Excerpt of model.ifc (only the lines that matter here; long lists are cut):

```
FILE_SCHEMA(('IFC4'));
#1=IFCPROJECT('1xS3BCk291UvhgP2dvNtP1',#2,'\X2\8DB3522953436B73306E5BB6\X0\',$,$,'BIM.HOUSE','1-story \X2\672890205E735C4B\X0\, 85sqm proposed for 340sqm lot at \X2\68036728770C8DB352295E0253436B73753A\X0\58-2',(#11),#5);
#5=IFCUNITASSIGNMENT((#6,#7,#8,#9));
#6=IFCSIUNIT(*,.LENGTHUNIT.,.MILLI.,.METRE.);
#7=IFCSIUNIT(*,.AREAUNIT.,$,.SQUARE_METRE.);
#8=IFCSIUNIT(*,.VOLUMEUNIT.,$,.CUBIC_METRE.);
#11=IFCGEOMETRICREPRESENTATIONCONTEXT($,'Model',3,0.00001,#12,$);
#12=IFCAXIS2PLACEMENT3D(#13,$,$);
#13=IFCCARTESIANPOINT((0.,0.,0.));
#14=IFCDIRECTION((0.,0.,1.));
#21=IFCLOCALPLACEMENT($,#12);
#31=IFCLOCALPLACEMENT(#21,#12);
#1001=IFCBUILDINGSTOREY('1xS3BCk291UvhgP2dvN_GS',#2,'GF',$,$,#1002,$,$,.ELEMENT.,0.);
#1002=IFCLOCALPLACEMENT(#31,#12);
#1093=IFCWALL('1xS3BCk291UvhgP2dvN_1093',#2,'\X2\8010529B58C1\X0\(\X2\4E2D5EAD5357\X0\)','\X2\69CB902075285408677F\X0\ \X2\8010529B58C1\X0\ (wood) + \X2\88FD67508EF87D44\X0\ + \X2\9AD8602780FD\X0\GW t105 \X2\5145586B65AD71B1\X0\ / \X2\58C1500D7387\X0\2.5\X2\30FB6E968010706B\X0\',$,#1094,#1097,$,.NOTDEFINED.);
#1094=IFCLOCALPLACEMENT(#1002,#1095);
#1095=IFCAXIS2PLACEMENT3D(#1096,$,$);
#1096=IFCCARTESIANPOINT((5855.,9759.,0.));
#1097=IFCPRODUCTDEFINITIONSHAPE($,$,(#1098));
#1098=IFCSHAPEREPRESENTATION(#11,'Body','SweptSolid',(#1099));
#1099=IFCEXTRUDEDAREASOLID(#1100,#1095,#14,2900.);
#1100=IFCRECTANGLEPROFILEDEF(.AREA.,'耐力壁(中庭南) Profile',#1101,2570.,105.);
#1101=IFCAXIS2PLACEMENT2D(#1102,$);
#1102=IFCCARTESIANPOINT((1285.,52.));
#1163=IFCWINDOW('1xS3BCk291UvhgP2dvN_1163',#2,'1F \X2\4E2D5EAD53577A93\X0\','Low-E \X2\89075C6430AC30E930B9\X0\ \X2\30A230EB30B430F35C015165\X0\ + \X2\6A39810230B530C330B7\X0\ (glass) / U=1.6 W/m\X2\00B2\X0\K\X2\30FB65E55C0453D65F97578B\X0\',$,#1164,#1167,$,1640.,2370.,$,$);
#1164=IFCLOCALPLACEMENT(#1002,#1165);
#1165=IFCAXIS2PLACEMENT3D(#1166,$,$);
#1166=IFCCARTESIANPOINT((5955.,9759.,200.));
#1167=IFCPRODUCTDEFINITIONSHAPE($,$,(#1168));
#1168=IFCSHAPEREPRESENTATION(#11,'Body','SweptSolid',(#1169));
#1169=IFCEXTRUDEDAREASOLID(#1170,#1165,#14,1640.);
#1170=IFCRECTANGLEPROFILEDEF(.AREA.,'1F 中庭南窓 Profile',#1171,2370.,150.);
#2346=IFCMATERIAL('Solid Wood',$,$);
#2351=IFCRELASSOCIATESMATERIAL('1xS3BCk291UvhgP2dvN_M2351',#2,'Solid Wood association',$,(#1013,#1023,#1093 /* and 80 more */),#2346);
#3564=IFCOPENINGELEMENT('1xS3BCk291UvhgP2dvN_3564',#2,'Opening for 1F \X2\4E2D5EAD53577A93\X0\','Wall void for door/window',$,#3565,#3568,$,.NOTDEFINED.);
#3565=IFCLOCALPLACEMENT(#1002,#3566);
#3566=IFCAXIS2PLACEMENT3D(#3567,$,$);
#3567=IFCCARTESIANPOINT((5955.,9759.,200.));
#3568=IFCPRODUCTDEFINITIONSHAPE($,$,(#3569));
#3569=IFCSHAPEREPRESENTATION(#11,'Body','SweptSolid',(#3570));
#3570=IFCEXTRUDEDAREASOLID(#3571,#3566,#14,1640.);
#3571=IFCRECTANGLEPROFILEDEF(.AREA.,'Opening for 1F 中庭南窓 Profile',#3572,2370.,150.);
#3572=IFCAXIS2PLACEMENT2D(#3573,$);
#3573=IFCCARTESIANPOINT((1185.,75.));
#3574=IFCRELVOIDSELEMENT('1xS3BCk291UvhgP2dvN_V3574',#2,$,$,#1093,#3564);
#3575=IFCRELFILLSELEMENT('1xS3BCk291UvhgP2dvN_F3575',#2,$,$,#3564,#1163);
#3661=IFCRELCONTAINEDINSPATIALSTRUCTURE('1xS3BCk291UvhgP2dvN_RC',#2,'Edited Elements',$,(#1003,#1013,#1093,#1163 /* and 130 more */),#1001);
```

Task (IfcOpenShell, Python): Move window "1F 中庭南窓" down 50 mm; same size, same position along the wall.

```python
import numpy as np
import ifcopenshell
import ifcopenshell.api.geometry
import ifcopenshell.util.placement
import ifcopenshell.util.unit

model = ifcopenshell.open("model.ifc")
unit_scale = ifcopenshell.util.unit.calculate_unit_scale(model)

window = model.by_guid("1xS3BCk291UvhgP2dvN_1163")
opening = window.FillsVoids[0].RelatingOpeningElement
dz = -50.0

shift = np.array([0.0, 0.0, dz])
# The window is not placed relative to its opening, so move both.
for product in (opening, window):
    matrix = ifcopenshell.util.placement.get_local_placement(product.ObjectPlacement)
    matrix[:3, 3] += shift
    ifcopenshell.api.geometry.edit_object_placement(model, product=product, matrix=matrix, is_si=False)

print(f"moved by {dz * unit_scale:+.3f} m")

model.write("model_rev.ifc")
```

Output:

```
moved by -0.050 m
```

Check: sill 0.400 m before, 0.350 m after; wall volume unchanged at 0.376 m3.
